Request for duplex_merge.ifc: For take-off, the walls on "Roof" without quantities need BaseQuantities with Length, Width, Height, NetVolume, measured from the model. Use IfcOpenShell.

First a look at what the model holds.

```python
import ifcopenshell
import ifcopenshell.util.element
import ifcopenshell.util.unit

model = ifcopenshell.open("duplex_merge.ifc")
print(model.schema)
for unit_type in ("LENGTHUNIT", "AREAUNIT", "VOLUMEUNIT"):
    print(unit_type, ifcopenshell.util.unit.calculate_unit_scale(model, unit_type))
storey = next(s for s in model.by_type("IfcBuildingStorey") if s.Name == "Roof")
walls = [e for e in ifcopenshell.util.element.get_decomposition(storey) if e.is_a("IfcWall")]
for e in sorted(walls, key=lambda e: e.id()):
    print(e.id(), e.is_a(), e.Name, list(ifcopenshell.util.element.get_psets(e, qtos_only=True)), sep=" | ")
```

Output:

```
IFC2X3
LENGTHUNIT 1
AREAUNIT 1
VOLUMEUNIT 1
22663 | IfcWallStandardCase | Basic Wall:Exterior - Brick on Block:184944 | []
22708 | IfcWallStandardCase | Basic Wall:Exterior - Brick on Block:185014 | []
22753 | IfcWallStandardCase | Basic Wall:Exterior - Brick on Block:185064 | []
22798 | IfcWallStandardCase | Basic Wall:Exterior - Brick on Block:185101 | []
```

```python
import ifcopenshell
import ifcopenshell.api.pset
import ifcopenshell.geom
import ifcopenshell.util.element
import ifcopenshell.util.shape
import ifcopenshell.util.unit

model = ifcopenshell.open("duplex_merge.ifc")
unit_scale = ifcopenshell.util.unit.calculate_unit_scale(model)
volume_scale = ifcopenshell.util.unit.calculate_unit_scale(model, "VOLUMEUNIT")
settings = ifcopenshell.geom.settings()

storey = next(s for s in model.by_type("IfcBuildingStorey") if s.Name == "Roof")
walls = [e for e in ifcopenshell.util.element.get_decomposition(storey) if e.is_a("IfcWall")]

for e in sorted(walls, key=lambda e: e.id()):
    if ifcopenshell.util.element.get_psets(e, qtos_only=True, should_inherit=False):
        continue
    # Geometry comes back in metres, in the element's own axes.
    shape = ifcopenshell.geom.create_shape(settings, e)
    values = {
        "Length": ifcopenshell.util.shape.get_x(shape.geometry) / unit_scale,
        "Width": ifcopenshell.util.shape.get_y(shape.geometry) / unit_scale,
        "Height": ifcopenshell.util.shape.get_z(shape.geometry) / unit_scale,
        "NetVolume": ifcopenshell.util.shape.get_volume(shape.geometry) / volume_scale,
    }
    qto = ifcopenshell.api.pset.add_qto(model, product=e, name="BaseQuantities")
    ifcopenshell.api.pset.edit_qto(model, qto=qto, properties=values)
    print(e.id(), {k: round(v, 3) for k, v in values.items()})

model.write("duplex_merge_updated.ifc")
```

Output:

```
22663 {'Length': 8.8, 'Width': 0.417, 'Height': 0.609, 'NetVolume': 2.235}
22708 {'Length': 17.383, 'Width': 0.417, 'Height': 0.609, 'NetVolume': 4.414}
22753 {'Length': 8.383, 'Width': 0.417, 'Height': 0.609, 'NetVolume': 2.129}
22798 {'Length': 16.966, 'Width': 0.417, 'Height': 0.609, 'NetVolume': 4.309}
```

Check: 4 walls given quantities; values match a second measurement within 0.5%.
